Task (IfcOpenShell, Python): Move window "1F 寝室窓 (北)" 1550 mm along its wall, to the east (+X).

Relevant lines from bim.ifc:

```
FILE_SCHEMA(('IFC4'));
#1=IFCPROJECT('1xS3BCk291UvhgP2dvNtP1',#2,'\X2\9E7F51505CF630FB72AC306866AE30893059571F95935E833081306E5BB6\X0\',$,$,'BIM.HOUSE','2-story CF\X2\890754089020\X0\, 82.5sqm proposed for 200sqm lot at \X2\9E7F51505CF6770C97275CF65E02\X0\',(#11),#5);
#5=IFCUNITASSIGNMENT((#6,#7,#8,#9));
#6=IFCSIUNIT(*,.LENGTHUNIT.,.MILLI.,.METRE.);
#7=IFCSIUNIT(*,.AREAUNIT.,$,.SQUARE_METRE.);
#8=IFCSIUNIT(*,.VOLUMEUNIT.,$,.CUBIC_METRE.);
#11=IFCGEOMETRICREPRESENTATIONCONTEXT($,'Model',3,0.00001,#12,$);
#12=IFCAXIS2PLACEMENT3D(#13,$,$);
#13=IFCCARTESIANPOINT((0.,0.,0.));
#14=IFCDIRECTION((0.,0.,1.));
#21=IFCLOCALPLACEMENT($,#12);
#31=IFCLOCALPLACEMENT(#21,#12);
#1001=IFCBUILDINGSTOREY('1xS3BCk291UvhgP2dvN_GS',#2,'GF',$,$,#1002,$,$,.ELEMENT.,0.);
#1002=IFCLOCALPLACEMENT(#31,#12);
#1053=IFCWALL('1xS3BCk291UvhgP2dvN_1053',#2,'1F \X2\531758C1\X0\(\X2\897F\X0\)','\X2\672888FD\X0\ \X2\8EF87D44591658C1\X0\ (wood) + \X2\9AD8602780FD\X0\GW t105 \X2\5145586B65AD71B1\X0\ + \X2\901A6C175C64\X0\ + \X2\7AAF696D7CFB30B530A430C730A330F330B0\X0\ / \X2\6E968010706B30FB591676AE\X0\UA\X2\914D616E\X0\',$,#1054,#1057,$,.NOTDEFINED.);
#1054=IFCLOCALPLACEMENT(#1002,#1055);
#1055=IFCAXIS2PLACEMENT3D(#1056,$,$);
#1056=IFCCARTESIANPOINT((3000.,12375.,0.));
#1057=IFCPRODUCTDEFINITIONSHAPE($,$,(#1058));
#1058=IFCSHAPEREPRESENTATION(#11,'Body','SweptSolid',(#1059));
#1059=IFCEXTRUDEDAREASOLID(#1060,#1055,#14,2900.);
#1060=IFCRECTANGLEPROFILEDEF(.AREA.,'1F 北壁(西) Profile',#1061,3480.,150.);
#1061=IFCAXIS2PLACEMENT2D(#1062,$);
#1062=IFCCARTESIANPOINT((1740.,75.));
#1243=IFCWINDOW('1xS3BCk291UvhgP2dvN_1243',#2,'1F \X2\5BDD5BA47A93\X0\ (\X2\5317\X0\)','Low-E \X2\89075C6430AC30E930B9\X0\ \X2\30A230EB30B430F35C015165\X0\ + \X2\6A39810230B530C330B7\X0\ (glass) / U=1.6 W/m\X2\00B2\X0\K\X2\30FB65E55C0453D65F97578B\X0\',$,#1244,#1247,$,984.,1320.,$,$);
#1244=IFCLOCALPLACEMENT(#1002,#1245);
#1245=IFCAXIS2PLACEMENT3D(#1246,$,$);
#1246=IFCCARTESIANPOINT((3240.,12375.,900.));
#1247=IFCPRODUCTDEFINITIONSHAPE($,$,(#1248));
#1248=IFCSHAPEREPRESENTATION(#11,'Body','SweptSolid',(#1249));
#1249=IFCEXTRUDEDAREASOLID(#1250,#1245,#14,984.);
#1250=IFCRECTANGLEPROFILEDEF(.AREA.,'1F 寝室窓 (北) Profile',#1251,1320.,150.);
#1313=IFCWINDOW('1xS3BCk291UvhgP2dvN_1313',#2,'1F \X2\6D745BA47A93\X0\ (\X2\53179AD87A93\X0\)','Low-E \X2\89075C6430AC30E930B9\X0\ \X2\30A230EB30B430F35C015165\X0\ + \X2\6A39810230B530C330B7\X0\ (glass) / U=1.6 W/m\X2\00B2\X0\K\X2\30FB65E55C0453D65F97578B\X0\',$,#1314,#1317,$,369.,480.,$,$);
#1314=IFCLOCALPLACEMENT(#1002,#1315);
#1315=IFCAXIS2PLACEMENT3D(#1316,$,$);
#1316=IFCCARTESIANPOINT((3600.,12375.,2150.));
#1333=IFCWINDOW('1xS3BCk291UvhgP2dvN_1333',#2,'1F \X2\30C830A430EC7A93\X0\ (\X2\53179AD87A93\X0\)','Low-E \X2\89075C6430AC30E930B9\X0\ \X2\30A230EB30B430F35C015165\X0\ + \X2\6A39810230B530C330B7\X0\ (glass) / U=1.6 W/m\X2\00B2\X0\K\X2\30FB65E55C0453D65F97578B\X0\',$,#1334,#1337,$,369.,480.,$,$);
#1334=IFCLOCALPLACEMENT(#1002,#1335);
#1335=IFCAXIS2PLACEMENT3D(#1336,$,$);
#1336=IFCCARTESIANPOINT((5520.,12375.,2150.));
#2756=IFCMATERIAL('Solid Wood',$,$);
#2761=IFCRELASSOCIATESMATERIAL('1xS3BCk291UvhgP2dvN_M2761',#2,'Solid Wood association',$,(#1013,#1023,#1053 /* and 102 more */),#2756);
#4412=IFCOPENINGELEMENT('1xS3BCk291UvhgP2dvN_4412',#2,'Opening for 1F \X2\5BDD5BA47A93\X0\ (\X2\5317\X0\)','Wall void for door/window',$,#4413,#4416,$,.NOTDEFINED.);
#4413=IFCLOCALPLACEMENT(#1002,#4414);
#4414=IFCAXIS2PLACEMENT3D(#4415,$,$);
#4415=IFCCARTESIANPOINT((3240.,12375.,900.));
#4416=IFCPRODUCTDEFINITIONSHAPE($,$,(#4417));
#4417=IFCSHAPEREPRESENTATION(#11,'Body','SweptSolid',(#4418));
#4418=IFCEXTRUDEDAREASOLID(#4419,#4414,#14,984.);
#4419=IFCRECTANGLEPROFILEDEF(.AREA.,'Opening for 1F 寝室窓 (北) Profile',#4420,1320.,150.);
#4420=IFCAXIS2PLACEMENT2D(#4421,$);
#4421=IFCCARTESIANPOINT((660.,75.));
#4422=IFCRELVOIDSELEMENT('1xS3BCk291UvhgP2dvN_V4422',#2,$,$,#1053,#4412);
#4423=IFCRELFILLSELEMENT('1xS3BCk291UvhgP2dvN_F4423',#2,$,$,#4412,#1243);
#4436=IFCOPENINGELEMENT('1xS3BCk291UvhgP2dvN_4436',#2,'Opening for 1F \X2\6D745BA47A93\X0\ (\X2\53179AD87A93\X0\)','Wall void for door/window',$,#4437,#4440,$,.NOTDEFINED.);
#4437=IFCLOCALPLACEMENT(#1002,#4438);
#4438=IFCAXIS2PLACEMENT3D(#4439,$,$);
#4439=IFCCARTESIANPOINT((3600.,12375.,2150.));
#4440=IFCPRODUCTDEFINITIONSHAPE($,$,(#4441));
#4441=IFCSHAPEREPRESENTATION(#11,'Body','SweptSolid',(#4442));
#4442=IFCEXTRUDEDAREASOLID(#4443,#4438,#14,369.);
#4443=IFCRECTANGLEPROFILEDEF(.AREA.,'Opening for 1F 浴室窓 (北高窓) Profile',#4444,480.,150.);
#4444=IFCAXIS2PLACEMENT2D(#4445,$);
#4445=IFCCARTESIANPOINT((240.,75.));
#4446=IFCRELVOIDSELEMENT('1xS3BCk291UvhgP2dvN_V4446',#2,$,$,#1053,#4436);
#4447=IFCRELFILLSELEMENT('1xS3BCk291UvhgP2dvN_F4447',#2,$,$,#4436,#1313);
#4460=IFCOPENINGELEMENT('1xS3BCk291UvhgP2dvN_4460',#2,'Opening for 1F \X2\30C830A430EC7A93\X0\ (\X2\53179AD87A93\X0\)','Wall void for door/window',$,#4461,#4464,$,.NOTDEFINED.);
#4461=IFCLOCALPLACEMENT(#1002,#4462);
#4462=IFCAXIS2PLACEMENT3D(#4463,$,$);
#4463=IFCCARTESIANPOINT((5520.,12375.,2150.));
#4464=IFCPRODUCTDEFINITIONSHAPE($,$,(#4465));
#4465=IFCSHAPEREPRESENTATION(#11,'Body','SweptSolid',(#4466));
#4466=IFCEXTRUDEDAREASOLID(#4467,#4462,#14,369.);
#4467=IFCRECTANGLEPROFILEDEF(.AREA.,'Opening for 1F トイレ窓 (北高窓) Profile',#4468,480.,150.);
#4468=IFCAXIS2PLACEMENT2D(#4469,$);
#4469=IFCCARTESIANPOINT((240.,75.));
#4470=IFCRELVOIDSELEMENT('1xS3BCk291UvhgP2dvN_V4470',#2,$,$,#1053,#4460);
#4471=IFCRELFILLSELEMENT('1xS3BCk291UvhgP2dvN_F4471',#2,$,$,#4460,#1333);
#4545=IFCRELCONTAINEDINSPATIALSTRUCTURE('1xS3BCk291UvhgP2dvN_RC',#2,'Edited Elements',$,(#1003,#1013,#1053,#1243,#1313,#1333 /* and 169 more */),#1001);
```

```python
import ifcopenshell
import ifcopenshell.api.geometry
import ifcopenshell.util.placement

model = ifcopenshell.open("bim.ifc")

window = model.by_guid("1xS3BCk291UvhgP2dvN_1243")
opening = window.FillsVoids[0].RelatingOpeningElement
wall = opening.VoidsElements[0].RelatingBuildingElement

wall_matrix = ifcopenshell.util.placement.get_local_placement(wall.ObjectPlacement)
shift = wall_matrix[:3, 0] * 1550.0
before = ifcopenshell.util.placement.get_local_placement(window.ObjectPlacement)[:3, 3].copy()

# The window is not placed relative to its opening, so move both.
for product in (opening, window):
    matrix = ifcopenshell.util.placement.get_local_placement(product.ObjectPlacement)
    matrix[:3, 3] += shift
    ifcopenshell.api.geometry.edit_object_placement(model, product=product, matrix=matrix, is_si=False)

after = ifcopenshell.util.placement.get_local_placement(window.ObjectPlacement)[:3, 3]
print("window moved by", (after - before).round(3) + 0.0)

model.write("bim_v2.ifc")
```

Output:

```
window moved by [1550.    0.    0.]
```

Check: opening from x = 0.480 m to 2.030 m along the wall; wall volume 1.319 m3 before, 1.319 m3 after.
